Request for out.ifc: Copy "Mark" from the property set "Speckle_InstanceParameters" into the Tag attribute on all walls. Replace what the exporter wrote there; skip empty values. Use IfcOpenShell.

First a look at what the model holds.

```python
import ifcopenshell
import ifcopenshell.util.element

model = ifcopenshell.open("out.ifc")
print(model.schema)
walls = model.by_type("IfcWall")
print(len(walls), "walls")
for e in walls[:8]:
    source = ifcopenshell.util.element.get_pset(e, "Speckle_InstanceParameters", "Mark")
    target = e.Tag
    print(e.id(), repr(source), repr(target), sep=" | ")
```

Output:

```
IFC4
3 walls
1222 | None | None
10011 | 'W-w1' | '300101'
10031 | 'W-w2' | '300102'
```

```python
import ifcopenshell
import ifcopenshell.util.element

model = ifcopenshell.open("out.ifc")

count = 0
for e in model.by_type("IfcWall"):
    value = ifcopenshell.util.element.get_pset(e, "Speckle_InstanceParameters", "Mark")
    current = e.Tag
    if not value or not value.strip() or current == value:
        continue
    e.Tag = value
    count += 1

print(count, "walls updated")

model.write("out_v2.ifc")
```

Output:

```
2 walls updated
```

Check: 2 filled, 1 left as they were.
